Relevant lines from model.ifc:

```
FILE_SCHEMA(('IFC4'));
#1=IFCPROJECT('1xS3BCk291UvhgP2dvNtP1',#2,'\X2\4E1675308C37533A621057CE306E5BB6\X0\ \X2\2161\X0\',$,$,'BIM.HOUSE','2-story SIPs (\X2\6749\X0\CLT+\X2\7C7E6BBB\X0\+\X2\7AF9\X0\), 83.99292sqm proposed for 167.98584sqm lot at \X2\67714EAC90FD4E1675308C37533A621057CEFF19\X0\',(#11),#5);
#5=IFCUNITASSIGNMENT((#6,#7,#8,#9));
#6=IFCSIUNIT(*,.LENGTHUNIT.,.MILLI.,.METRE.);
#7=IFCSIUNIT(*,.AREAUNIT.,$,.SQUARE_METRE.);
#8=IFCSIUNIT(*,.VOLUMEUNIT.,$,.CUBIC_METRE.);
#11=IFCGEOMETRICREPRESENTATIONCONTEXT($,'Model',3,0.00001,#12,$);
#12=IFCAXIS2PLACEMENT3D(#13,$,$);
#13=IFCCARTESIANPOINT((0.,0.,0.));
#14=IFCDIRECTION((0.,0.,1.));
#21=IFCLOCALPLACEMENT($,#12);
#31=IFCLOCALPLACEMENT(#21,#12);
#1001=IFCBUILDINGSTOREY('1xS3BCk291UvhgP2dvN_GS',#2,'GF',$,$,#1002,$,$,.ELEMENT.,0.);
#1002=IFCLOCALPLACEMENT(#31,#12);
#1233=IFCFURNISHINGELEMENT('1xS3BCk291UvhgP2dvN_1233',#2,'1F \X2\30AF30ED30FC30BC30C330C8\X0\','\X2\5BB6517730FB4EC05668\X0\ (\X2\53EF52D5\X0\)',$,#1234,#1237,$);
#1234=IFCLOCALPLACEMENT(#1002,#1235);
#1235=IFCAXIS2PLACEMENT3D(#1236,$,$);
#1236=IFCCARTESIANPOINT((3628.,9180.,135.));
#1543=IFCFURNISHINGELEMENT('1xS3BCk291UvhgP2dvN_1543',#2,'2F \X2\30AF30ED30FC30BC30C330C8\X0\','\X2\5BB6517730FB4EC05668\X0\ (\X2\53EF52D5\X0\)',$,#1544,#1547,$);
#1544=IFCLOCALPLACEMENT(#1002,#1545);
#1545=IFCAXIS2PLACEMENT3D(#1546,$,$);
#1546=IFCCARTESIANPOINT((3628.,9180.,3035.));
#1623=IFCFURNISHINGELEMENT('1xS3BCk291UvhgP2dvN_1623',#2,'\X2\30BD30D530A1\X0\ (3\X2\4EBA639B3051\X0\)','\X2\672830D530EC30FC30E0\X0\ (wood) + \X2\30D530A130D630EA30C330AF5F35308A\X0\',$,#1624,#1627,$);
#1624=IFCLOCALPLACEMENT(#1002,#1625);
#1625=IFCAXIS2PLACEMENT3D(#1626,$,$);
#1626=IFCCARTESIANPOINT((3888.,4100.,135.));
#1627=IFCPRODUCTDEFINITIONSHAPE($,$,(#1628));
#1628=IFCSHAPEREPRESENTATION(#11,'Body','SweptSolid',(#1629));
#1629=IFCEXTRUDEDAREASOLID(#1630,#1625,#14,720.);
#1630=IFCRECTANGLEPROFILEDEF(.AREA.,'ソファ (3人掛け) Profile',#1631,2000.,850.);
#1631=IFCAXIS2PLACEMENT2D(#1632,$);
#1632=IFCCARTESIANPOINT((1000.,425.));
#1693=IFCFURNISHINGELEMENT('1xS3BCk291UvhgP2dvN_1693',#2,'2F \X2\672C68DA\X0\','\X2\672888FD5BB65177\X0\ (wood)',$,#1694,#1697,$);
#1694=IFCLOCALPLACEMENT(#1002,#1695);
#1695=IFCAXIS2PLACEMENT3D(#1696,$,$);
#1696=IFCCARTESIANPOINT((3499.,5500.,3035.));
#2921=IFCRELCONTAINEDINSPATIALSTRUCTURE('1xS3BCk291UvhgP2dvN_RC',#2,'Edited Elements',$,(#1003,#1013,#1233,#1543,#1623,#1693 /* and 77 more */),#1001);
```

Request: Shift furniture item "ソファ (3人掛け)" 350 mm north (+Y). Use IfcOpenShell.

```python
import ifcopenshell
import ifcopenshell.api.geometry
import ifcopenshell.util.placement

model = ifcopenshell.open("model.ifc")

item = model.by_guid("1xS3BCk291UvhgP2dvN_1623")
matrix = ifcopenshell.util.placement.get_local_placement(item.ObjectPlacement)
matrix[1, 3] += 350.0
ifcopenshell.api.geometry.edit_object_placement(model, product=item, matrix=matrix, is_si=False)

print(ifcopenshell.util.placement.get_local_placement(item.ObjectPlacement).round(3) + 0.0)

model.write("model_edited.ifc")
```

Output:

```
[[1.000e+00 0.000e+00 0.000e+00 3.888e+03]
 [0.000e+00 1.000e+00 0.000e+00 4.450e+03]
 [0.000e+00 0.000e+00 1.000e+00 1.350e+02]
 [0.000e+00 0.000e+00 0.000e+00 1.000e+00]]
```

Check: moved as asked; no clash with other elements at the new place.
